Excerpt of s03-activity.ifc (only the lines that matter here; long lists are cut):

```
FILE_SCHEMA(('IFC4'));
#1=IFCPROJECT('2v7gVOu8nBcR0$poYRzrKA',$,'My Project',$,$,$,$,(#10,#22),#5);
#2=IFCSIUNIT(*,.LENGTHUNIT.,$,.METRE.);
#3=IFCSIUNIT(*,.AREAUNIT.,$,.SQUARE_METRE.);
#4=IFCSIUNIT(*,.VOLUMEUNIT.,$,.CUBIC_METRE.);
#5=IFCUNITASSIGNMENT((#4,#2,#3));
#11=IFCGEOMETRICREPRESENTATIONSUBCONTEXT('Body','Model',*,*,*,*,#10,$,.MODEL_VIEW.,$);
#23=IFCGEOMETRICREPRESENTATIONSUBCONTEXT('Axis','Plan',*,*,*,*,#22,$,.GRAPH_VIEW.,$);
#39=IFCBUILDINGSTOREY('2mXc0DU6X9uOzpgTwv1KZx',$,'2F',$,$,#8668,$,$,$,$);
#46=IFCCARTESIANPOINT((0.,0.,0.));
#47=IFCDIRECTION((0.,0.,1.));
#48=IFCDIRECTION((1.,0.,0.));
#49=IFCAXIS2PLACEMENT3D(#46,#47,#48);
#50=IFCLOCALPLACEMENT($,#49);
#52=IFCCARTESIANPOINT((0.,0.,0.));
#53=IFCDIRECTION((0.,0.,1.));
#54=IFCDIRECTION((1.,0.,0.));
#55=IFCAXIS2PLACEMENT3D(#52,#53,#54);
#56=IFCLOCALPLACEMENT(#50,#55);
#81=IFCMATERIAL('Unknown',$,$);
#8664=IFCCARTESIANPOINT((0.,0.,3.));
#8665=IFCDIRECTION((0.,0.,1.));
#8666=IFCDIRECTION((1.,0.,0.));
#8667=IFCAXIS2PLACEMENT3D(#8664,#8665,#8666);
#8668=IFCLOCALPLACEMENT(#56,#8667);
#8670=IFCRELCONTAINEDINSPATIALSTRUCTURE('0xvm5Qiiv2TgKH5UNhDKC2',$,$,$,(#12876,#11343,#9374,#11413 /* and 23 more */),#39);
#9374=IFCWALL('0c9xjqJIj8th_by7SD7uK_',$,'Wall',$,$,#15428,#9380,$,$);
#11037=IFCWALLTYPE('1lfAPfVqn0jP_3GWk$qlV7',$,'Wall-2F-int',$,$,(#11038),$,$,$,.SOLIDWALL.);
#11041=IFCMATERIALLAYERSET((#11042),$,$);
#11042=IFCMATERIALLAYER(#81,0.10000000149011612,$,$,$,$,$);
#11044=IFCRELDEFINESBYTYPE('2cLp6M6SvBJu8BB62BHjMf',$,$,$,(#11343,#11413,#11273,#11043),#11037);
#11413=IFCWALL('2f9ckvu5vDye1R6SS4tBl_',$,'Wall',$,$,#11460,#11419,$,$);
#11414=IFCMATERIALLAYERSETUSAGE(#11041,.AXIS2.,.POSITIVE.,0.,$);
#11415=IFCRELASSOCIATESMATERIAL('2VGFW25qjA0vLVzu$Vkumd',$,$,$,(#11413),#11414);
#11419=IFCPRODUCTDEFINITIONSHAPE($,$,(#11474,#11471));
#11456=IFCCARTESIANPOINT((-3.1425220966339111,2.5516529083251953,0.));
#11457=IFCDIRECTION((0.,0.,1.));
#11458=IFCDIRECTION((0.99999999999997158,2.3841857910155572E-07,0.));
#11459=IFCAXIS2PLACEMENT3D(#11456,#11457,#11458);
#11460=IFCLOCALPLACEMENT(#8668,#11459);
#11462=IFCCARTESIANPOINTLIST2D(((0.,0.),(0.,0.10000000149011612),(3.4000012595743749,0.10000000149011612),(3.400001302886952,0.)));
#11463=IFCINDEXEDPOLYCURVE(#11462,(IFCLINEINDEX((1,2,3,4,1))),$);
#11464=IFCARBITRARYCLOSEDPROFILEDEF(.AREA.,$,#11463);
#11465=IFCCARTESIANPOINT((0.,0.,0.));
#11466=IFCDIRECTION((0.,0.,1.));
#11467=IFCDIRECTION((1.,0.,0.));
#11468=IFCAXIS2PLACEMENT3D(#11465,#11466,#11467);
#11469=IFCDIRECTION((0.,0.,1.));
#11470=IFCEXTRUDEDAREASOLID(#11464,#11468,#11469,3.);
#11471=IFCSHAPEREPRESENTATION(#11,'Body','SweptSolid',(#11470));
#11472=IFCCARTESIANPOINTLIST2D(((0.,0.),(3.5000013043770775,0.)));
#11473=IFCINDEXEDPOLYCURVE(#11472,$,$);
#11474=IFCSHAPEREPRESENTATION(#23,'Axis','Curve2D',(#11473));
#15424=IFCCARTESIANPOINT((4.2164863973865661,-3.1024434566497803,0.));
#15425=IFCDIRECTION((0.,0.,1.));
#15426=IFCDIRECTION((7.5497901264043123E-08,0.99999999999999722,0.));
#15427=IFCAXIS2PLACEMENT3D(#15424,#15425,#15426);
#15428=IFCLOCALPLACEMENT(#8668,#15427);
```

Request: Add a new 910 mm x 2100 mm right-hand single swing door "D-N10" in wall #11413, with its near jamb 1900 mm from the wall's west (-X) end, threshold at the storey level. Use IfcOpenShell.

```python
import numpy as np
import ifcopenshell
import ifcopenshell.api.feature
import ifcopenshell.api.geometry
import ifcopenshell.api.root
import ifcopenshell.api.spatial
import ifcopenshell.geom
import ifcopenshell.util.element
import ifcopenshell.util.placement
import ifcopenshell.util.representation
import ifcopenshell.util.shape
import ifcopenshell.util.unit

model = ifcopenshell.open("s03-activity.ifc")
unit_scale = ifcopenshell.util.unit.calculate_unit_scale(model)
settings = ifcopenshell.geom.settings()


def volume(element):
    """Net volume in cubic metres, openings subtracted."""
    shape = ifcopenshell.geom.create_shape(settings, element)
    return ifcopenshell.util.shape.get_volume(shape.geometry)


wall = model.by_guid("2f9ckvu5vDye1R6SS4tBl_")
storey = ifcopenshell.util.element.get_container(wall, ifc_class="IfcBuildingStorey")
context = ifcopenshell.util.representation.get_context(model, "Model", "Body", "MODEL_VIEW")
before = volume(wall)

width, height, from_end, sill = 0.91, 2.1, 1.9, 0.0  # metres

# The wall runs along its own X axis, and the end named is its -X end.
wall_shape = ifcopenshell.geom.create_shape(settings, wall)
x, y, z = ifcopenshell.util.shape.get_vertices(wall_shape.geometry).T
start = x.min() + from_end
face, thickness = float(y.min()), float(y.max() - y.min())
wall_matrix = ifcopenshell.util.placement.get_local_placement(wall.ObjectPlacement)
level = ifcopenshell.util.placement.get_local_placement(storey.ObjectPlacement)[2, 3]


def in_wall(x, y):
    """Placement at x, y metres in the wall's axes, at sill height."""
    matrix = wall_matrix.copy()
    matrix[:, 3] = wall_matrix @ np.array([x / unit_scale, y / unit_scale, 0.0, 1.0])
    matrix[2, 3] = level + sill / unit_scale
    return matrix


# Opening: a box that overshoots both wall faces by 50 mm.
opening = ifcopenshell.api.root.create_entity(model, ifc_class="IfcOpeningElement", predefined_type="OPENING")
box = ifcopenshell.api.geometry.add_wall_representation(
    model, context=context, length=width, height=height, thickness=thickness + 0.1
)
ifcopenshell.api.geometry.assign_representation(model, product=opening, representation=box)
ifcopenshell.api.geometry.edit_object_placement(model, product=opening, matrix=in_wall(start, face - 0.05), is_si=False)
ifcopenshell.api.feature.add_feature(model, feature=opening, element=wall)

door = ifcopenshell.api.root.create_entity(model, ifc_class="IfcDoor", name="D-N10", predefined_type="DOOR")
door.OverallWidth, door.OverallHeight = width / unit_scale, height / unit_scale
door.OperationType = "SINGLE_SWING_RIGHT"
body = ifcopenshell.api.geometry.add_door_representation(
    model,
    context=context,
    overall_width=door.OverallWidth,
    overall_height=door.OverallHeight,
    operation_type="SINGLE_SWING_RIGHT",
    lining_properties={"LiningDepth": thickness / unit_scale, "ThresholdDepth": thickness / unit_scale},
)
ifcopenshell.api.geometry.assign_representation(model, product=door, representation=body)
ifcopenshell.api.spatial.assign_container(model, products=[door], relating_structure=storey)
ifcopenshell.api.feature.add_filling(model, opening=opening, element=door)

# The lining spans the wall, so the door starts at the wall face.
ifcopenshell.api.geometry.edit_object_placement(model, product=door, matrix=in_wall(start, face), is_si=False)

after = volume(wall)

print(f"wall volume {before:.3f} -> {after:.3f} m3")

model.write("s03-activity_updated.ifc")
```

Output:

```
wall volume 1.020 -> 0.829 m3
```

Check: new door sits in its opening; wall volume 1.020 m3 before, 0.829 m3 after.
